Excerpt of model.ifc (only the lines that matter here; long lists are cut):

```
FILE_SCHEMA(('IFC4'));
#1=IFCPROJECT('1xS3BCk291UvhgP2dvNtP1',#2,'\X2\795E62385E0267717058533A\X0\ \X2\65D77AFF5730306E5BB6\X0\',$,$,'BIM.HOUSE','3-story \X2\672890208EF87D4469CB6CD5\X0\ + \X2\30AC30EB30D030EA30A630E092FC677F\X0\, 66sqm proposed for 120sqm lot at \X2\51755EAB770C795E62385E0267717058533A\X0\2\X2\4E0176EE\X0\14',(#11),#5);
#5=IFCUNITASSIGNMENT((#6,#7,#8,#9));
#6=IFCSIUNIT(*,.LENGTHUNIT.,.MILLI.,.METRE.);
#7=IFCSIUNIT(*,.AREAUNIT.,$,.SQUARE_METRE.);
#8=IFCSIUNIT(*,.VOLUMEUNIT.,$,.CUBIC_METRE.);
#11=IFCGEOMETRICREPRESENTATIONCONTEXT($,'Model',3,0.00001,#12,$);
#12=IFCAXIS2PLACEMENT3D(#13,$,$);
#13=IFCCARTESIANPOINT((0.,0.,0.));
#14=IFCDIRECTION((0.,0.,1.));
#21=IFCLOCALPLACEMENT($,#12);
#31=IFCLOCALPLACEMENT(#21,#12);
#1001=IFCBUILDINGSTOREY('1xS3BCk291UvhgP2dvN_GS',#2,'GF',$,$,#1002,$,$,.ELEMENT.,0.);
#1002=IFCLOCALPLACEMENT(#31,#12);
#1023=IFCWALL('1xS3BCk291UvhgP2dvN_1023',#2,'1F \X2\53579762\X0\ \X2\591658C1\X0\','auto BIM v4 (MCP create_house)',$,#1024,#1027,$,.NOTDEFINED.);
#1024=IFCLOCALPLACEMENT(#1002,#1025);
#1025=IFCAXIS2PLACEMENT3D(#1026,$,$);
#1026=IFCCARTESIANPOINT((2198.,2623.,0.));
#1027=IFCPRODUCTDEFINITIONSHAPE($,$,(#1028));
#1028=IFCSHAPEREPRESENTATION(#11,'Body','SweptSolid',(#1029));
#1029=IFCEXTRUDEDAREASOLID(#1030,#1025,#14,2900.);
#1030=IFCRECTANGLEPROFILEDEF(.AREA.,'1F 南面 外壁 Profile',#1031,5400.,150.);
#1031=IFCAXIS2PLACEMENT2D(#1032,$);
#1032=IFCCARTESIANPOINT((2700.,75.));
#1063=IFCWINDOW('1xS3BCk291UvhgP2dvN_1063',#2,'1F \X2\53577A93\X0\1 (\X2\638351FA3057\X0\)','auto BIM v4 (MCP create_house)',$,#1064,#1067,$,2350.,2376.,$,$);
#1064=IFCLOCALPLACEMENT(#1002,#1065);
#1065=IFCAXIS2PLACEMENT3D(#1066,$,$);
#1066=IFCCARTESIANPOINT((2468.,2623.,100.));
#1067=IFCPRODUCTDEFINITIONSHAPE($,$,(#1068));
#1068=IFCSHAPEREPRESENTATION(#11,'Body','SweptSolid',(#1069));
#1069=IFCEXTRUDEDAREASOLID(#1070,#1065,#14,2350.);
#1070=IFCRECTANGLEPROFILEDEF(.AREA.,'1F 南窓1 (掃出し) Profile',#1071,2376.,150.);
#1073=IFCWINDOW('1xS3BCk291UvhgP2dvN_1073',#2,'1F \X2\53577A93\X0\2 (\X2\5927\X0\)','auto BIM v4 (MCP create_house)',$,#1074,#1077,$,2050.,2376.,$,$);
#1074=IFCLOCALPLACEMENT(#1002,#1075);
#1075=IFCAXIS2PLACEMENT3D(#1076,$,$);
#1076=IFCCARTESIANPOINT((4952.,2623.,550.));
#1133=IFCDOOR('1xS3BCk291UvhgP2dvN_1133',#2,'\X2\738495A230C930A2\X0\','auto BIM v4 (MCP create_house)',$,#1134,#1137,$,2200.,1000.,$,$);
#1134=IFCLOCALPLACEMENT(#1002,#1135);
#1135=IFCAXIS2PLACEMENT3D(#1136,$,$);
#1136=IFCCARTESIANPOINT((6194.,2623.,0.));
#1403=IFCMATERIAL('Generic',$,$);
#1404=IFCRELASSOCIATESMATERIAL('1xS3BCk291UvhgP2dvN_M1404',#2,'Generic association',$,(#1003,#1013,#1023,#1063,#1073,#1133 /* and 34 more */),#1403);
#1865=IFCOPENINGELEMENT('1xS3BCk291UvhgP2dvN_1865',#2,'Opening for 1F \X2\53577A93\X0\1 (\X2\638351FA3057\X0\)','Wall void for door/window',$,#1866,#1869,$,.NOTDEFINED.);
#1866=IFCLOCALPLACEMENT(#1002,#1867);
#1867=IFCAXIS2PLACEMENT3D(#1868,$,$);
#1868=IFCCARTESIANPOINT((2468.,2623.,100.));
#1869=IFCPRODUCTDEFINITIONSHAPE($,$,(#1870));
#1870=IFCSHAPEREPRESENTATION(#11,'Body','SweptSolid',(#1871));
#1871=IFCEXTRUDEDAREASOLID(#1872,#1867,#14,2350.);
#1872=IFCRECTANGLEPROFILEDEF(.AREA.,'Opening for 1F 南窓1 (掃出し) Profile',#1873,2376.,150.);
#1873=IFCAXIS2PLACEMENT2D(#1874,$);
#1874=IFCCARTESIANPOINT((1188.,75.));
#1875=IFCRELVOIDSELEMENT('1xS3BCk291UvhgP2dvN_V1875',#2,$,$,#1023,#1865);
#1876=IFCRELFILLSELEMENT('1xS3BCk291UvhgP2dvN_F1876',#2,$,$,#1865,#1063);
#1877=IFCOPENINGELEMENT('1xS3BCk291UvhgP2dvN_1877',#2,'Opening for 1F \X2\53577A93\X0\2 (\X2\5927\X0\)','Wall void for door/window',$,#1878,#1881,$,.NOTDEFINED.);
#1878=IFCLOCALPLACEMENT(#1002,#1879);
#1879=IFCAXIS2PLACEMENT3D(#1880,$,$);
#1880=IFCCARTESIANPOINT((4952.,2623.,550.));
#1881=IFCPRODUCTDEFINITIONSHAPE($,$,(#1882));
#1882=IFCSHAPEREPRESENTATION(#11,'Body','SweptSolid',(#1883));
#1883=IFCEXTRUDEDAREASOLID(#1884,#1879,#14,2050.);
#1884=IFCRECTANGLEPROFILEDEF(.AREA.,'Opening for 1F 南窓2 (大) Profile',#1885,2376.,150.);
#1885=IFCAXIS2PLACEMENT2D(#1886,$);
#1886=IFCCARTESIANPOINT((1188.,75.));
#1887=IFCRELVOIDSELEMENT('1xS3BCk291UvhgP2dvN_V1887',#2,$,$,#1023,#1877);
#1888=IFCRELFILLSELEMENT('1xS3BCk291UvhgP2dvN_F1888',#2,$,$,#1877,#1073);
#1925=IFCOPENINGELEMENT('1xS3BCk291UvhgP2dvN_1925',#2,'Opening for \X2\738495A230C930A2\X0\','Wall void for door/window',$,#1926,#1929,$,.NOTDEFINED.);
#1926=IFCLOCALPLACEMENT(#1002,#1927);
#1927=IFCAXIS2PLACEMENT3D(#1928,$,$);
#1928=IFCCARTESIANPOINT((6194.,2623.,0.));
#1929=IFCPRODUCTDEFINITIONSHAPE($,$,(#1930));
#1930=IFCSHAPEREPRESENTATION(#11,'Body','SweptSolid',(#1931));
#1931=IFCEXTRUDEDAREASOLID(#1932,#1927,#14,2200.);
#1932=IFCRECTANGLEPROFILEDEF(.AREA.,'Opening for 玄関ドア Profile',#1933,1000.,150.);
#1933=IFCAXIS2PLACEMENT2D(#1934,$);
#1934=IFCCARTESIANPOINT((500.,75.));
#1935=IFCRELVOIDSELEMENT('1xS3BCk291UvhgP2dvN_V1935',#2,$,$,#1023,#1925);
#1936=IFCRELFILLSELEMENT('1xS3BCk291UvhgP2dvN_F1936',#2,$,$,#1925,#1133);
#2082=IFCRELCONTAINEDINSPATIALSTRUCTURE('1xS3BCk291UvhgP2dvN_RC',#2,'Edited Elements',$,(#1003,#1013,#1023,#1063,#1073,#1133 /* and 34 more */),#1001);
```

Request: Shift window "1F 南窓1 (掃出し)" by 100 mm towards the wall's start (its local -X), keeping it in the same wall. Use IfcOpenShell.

```python
import ifcopenshell
import ifcopenshell.api.geometry
import ifcopenshell.util.placement

model = ifcopenshell.open("model.ifc")

window = model.by_guid("1xS3BCk291UvhgP2dvN_1063")
opening = window.FillsVoids[0].RelatingOpeningElement
wall = opening.VoidsElements[0].RelatingBuildingElement

wall_matrix = ifcopenshell.util.placement.get_local_placement(wall.ObjectPlacement)
shift = wall_matrix[:3, 0] * -100.0
before = ifcopenshell.util.placement.get_local_placement(window.ObjectPlacement)[:3, 3].copy()

# The window is not placed relative to its opening, so move both.
for product in (opening, window):
    matrix = ifcopenshell.util.placement.get_local_placement(product.ObjectPlacement)
    matrix[:3, 3] += shift
    ifcopenshell.api.geometry.edit_object_placement(model, product=product, matrix=matrix, is_si=False)

after = ifcopenshell.util.placement.get_local_placement(window.ObjectPlacement)[:3, 3]
print("window moved by", (after - before).round(3) + 0.0)

model.write("model_updated.ifc")
```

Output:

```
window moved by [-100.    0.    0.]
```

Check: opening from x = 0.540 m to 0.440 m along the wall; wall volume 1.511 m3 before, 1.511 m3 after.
